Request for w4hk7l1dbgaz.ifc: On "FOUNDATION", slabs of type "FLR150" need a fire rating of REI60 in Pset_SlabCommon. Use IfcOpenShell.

First a look at what the model holds.

```python
import ifcopenshell
import ifcopenshell.util.element

model = ifcopenshell.open("w4hk7l1dbgaz.ifc")
print(model.schema)
storey = next(s for s in model.by_type("IfcBuildingStorey") if s.Name == "FOUNDATION")
slabs = [e for e in ifcopenshell.util.element.get_decomposition(storey) if e.is_a("IfcSlab")]
seen = {}
for e in slabs:
    element_type = ifcopenshell.util.element.get_type(e)
    key = (element_type.Name if element_type != e and element_type else None, ifcopenshell.util.element.get_pset(e, "Pset_SlabCommon", "FireRating"))
    seen[key] = seen.get(key, 0) + 1
for (name, value), count in sorted(seen.items(), key=str):
    print(count, "x", name, "|", value)
```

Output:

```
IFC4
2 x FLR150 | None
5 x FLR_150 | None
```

```python
import ifcopenshell
import ifcopenshell.api.pset
import ifcopenshell.util.element

model = ifcopenshell.open("w4hk7l1dbgaz.ifc")

storey = next(s for s in model.by_type("IfcBuildingStorey") if s.Name == "FOUNDATION")
slabs = [e for e in ifcopenshell.util.element.get_decomposition(storey) if e.is_a("IfcSlab")]

count = 0
for e in slabs:
    element_type = ifcopenshell.util.element.get_type(e)
    if element_type in (None, e) or element_type.Name != "FLR150":
        continue
    # add_pset returns the element's existing set when there is one.
    pset = ifcopenshell.api.pset.add_pset(model, product=e, name="Pset_SlabCommon")
    ifcopenshell.api.pset.edit_pset(model, pset=pset, properties={"FireRating": "REI60"})
    count += 1

print(count, "slabs updated")

model.write("w4hk7l1dbgaz_v2.ifc")
```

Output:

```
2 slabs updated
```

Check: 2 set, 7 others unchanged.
